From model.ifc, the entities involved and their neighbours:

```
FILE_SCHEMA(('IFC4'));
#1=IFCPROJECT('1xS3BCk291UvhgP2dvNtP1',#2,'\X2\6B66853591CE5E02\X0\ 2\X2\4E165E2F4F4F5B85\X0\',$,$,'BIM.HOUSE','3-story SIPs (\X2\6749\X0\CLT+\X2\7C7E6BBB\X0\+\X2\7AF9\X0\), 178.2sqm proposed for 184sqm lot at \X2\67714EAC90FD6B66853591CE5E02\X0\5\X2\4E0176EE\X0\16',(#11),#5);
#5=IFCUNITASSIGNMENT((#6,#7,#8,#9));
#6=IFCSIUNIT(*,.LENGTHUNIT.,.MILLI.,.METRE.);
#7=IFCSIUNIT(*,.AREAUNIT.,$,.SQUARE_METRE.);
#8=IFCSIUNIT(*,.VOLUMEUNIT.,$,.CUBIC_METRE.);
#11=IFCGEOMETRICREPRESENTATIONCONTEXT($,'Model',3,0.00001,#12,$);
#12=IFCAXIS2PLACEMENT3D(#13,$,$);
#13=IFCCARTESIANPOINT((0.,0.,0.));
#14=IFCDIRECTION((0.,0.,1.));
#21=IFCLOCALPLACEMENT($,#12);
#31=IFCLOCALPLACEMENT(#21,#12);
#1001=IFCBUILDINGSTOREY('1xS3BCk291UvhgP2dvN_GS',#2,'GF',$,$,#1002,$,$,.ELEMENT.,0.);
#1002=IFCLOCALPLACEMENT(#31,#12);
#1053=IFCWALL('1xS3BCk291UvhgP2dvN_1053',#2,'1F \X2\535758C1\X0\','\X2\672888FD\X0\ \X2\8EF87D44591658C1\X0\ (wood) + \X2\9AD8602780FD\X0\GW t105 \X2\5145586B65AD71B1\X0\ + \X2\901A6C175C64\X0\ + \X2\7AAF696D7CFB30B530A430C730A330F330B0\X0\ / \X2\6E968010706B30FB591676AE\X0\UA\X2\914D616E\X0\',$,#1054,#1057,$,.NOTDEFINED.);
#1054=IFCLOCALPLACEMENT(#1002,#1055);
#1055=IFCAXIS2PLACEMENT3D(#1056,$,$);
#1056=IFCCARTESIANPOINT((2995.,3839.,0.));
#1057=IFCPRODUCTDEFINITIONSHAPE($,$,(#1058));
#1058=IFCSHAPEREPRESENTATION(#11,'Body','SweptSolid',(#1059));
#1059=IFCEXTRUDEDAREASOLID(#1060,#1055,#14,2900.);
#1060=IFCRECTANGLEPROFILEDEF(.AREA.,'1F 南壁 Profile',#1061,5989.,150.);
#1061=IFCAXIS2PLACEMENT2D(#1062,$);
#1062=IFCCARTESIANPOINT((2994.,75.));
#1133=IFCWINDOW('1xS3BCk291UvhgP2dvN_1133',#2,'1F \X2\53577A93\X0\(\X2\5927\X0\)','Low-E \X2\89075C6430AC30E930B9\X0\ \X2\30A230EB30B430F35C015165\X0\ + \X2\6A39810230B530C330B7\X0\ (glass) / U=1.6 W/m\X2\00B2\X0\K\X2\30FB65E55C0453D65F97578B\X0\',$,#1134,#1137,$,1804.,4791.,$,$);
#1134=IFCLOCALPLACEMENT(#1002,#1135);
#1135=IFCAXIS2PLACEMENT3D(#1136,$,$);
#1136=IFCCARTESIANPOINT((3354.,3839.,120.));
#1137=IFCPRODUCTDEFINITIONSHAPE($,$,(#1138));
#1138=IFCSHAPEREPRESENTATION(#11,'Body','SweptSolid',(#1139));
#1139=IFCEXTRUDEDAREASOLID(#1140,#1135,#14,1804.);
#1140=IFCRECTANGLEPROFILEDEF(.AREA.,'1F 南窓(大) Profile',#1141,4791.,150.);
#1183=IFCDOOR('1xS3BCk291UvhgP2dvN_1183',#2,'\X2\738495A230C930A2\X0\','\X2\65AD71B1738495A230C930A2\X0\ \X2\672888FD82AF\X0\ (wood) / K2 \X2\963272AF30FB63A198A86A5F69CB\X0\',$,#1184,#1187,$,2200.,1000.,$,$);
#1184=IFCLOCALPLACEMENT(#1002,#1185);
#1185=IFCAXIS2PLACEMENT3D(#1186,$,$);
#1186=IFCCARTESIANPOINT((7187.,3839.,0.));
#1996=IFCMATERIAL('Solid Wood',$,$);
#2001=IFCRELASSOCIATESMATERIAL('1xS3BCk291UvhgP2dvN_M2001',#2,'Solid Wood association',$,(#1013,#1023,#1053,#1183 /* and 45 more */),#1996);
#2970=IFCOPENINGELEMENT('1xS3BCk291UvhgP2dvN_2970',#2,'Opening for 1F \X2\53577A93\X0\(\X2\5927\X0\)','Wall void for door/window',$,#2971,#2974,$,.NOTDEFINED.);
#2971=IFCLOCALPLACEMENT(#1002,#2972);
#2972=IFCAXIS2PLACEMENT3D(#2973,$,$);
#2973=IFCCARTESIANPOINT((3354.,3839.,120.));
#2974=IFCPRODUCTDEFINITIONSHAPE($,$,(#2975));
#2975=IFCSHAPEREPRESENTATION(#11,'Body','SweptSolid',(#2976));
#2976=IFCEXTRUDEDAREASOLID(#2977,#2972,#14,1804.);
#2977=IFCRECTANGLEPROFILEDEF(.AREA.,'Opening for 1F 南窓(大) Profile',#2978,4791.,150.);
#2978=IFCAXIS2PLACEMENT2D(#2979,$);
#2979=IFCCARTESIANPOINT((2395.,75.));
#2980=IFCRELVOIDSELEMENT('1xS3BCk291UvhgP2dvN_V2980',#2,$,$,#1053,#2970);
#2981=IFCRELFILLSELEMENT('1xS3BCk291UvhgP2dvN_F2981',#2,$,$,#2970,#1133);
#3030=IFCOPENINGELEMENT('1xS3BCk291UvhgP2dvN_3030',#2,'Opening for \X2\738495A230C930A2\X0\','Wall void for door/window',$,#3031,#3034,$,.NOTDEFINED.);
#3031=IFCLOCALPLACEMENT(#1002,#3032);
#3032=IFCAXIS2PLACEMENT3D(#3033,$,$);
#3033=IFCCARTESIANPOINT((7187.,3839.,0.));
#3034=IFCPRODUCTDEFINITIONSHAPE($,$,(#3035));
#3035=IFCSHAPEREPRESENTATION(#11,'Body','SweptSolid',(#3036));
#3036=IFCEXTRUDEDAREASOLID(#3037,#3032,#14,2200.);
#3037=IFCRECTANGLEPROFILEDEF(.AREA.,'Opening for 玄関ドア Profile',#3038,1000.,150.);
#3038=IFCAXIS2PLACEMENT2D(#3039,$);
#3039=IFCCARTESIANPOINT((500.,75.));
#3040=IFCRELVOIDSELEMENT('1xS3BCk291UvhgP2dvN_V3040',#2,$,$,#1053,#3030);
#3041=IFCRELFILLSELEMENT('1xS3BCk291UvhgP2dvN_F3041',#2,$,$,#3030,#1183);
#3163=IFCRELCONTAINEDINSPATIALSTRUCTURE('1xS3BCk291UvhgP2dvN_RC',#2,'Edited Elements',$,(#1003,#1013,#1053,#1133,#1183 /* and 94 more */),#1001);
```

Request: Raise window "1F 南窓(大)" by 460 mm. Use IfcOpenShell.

```python
import numpy as np
import ifcopenshell
import ifcopenshell.api.geometry
import ifcopenshell.util.placement
import ifcopenshell.util.unit

model = ifcopenshell.open("model.ifc")
unit_scale = ifcopenshell.util.unit.calculate_unit_scale(model)

window = model.by_guid("1xS3BCk291UvhgP2dvN_1133")
opening = window.FillsVoids[0].RelatingOpeningElement
dz = 0.46 / unit_scale

shift = np.array([0.0, 0.0, dz])
# The window is not placed relative to its opening, so move both.
for product in (opening, window):
    matrix = ifcopenshell.util.placement.get_local_placement(product.ObjectPlacement)
    matrix[:3, 3] += shift
    ifcopenshell.api.geometry.edit_object_placement(model, product=product, matrix=matrix, is_si=False)

print(f"moved by {dz * unit_scale:+.3f} m")

model.write("model_rev.ifc")
```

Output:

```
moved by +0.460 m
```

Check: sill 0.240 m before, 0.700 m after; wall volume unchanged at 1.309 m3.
